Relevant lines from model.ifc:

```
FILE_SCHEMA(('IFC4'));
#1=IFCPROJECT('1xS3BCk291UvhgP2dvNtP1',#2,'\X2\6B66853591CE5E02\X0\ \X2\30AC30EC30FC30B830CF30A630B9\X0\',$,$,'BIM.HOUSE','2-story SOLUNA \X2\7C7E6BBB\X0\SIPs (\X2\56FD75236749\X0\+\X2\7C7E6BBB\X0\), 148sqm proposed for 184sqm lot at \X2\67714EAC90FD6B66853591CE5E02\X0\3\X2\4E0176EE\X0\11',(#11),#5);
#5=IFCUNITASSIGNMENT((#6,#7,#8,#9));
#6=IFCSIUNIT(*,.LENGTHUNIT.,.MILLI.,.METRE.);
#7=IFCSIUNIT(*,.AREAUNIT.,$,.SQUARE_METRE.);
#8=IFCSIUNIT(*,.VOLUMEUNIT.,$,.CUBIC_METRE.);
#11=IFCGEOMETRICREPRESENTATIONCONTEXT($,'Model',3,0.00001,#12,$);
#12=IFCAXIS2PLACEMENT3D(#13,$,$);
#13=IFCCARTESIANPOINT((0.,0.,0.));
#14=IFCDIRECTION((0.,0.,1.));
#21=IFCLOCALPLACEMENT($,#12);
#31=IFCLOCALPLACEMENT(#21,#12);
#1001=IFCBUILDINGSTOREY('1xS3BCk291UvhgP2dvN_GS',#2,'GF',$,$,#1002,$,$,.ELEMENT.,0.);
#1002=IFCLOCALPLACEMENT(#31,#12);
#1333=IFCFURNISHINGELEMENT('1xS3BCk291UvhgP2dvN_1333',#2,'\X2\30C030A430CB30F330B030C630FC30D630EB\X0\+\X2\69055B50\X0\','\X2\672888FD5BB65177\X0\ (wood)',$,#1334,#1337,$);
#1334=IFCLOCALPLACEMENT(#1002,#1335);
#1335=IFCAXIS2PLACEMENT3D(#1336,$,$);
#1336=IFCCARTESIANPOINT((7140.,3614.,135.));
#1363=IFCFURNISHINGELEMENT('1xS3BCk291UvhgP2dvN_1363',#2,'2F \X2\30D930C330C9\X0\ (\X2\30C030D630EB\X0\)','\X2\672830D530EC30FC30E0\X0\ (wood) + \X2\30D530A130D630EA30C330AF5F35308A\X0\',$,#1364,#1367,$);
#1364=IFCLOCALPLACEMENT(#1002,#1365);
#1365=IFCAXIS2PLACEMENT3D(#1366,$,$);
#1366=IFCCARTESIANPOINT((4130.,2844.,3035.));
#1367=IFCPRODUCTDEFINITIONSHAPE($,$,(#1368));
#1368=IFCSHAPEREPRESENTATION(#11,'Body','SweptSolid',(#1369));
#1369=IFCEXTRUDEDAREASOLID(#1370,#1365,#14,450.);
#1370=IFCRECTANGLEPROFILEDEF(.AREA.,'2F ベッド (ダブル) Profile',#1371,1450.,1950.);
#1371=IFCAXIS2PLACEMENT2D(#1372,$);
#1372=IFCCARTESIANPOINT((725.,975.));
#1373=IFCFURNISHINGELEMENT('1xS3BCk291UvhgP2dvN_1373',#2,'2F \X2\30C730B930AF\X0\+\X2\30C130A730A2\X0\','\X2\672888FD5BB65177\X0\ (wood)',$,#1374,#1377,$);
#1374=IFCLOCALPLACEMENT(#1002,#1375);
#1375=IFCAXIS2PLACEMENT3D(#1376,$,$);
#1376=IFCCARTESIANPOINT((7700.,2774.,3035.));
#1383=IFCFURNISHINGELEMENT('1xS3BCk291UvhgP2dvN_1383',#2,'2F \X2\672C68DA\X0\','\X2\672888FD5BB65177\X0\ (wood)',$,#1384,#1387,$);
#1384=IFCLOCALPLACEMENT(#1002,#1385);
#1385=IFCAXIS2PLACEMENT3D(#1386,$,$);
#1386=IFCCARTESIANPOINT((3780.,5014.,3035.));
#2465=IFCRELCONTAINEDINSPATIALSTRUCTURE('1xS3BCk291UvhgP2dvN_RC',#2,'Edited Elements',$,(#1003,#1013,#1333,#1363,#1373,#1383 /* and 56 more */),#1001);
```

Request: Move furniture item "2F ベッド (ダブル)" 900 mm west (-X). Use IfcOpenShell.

```python
import ifcopenshell
import ifcopenshell.api.geometry
import ifcopenshell.util.placement
import ifcopenshell.util.unit

model = ifcopenshell.open("model.ifc")
unit_scale = ifcopenshell.util.unit.calculate_unit_scale(model)

item = model.by_guid("1xS3BCk291UvhgP2dvN_1363")
matrix = ifcopenshell.util.placement.get_local_placement(item.ObjectPlacement)
matrix[0, 3] -= 0.9 / unit_scale
ifcopenshell.api.geometry.edit_object_placement(model, product=item, matrix=matrix, is_si=False)

print(ifcopenshell.util.placement.get_local_placement(item.ObjectPlacement).round(3) + 0.0)

model.write("model_rev.ifc")
```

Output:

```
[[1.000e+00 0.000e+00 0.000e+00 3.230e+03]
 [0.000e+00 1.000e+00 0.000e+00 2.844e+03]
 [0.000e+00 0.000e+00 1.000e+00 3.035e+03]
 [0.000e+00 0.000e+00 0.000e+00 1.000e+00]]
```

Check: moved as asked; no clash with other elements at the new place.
